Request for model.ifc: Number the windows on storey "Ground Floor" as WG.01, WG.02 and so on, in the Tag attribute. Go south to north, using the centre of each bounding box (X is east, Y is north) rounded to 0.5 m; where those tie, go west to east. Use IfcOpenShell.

First a look at what the model holds.

```python
import ifcopenshell
import ifcopenshell.util.element
import ifcopenshell.util.placement

model = ifcopenshell.open("model.ifc")
print(model.schema)
storey = next(s for s in model.by_type("IfcBuildingStorey") if s.Name == "Ground Floor")
windows = [e for e in ifcopenshell.util.element.get_decomposition(storey) if e.is_a("IfcWindow")]
for e in sorted(windows, key=lambda e: e.id()):
    origin = ifcopenshell.util.placement.get_local_placement(e.ObjectPlacement)[:3, 3]
    print(e.id(), e.Tag, e.Name, origin.round(2) + 0.0, sep=" | ")
```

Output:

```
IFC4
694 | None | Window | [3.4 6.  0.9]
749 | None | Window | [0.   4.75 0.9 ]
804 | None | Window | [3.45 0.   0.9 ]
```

```python
import ifcopenshell
import ifcopenshell.geom
import ifcopenshell.util.element
import ifcopenshell.util.shape

model = ifcopenshell.open("model.ifc")
settings = ifcopenshell.geom.settings()
settings.set("use-world-coords", True)


def centre(element):
    shape = ifcopenshell.geom.create_shape(settings, element)
    return ifcopenshell.util.shape.get_bbox_centroid(shape.geometry)


storey = next(s for s in model.by_type("IfcBuildingStorey") if s.Name == "Ground Floor")
windows = [e for e in ifcopenshell.util.element.get_decomposition(storey) if e.is_a("IfcWindow")]

# Insertion points can sit at a corner or the storey origin, so sort by the geometry (in metres).
centres = {e: centre(e) for e in windows}
windows.sort(key=lambda e: (round(centres[e][1] / 0.5), centres[e][0]))

for i, e in enumerate(windows, start=1):
    number = f"WG.{i:02d}"
    e.Tag = number
    print(e.id(), number)

model.write("model_v2.ifc")
```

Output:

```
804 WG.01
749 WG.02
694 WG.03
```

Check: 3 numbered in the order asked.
